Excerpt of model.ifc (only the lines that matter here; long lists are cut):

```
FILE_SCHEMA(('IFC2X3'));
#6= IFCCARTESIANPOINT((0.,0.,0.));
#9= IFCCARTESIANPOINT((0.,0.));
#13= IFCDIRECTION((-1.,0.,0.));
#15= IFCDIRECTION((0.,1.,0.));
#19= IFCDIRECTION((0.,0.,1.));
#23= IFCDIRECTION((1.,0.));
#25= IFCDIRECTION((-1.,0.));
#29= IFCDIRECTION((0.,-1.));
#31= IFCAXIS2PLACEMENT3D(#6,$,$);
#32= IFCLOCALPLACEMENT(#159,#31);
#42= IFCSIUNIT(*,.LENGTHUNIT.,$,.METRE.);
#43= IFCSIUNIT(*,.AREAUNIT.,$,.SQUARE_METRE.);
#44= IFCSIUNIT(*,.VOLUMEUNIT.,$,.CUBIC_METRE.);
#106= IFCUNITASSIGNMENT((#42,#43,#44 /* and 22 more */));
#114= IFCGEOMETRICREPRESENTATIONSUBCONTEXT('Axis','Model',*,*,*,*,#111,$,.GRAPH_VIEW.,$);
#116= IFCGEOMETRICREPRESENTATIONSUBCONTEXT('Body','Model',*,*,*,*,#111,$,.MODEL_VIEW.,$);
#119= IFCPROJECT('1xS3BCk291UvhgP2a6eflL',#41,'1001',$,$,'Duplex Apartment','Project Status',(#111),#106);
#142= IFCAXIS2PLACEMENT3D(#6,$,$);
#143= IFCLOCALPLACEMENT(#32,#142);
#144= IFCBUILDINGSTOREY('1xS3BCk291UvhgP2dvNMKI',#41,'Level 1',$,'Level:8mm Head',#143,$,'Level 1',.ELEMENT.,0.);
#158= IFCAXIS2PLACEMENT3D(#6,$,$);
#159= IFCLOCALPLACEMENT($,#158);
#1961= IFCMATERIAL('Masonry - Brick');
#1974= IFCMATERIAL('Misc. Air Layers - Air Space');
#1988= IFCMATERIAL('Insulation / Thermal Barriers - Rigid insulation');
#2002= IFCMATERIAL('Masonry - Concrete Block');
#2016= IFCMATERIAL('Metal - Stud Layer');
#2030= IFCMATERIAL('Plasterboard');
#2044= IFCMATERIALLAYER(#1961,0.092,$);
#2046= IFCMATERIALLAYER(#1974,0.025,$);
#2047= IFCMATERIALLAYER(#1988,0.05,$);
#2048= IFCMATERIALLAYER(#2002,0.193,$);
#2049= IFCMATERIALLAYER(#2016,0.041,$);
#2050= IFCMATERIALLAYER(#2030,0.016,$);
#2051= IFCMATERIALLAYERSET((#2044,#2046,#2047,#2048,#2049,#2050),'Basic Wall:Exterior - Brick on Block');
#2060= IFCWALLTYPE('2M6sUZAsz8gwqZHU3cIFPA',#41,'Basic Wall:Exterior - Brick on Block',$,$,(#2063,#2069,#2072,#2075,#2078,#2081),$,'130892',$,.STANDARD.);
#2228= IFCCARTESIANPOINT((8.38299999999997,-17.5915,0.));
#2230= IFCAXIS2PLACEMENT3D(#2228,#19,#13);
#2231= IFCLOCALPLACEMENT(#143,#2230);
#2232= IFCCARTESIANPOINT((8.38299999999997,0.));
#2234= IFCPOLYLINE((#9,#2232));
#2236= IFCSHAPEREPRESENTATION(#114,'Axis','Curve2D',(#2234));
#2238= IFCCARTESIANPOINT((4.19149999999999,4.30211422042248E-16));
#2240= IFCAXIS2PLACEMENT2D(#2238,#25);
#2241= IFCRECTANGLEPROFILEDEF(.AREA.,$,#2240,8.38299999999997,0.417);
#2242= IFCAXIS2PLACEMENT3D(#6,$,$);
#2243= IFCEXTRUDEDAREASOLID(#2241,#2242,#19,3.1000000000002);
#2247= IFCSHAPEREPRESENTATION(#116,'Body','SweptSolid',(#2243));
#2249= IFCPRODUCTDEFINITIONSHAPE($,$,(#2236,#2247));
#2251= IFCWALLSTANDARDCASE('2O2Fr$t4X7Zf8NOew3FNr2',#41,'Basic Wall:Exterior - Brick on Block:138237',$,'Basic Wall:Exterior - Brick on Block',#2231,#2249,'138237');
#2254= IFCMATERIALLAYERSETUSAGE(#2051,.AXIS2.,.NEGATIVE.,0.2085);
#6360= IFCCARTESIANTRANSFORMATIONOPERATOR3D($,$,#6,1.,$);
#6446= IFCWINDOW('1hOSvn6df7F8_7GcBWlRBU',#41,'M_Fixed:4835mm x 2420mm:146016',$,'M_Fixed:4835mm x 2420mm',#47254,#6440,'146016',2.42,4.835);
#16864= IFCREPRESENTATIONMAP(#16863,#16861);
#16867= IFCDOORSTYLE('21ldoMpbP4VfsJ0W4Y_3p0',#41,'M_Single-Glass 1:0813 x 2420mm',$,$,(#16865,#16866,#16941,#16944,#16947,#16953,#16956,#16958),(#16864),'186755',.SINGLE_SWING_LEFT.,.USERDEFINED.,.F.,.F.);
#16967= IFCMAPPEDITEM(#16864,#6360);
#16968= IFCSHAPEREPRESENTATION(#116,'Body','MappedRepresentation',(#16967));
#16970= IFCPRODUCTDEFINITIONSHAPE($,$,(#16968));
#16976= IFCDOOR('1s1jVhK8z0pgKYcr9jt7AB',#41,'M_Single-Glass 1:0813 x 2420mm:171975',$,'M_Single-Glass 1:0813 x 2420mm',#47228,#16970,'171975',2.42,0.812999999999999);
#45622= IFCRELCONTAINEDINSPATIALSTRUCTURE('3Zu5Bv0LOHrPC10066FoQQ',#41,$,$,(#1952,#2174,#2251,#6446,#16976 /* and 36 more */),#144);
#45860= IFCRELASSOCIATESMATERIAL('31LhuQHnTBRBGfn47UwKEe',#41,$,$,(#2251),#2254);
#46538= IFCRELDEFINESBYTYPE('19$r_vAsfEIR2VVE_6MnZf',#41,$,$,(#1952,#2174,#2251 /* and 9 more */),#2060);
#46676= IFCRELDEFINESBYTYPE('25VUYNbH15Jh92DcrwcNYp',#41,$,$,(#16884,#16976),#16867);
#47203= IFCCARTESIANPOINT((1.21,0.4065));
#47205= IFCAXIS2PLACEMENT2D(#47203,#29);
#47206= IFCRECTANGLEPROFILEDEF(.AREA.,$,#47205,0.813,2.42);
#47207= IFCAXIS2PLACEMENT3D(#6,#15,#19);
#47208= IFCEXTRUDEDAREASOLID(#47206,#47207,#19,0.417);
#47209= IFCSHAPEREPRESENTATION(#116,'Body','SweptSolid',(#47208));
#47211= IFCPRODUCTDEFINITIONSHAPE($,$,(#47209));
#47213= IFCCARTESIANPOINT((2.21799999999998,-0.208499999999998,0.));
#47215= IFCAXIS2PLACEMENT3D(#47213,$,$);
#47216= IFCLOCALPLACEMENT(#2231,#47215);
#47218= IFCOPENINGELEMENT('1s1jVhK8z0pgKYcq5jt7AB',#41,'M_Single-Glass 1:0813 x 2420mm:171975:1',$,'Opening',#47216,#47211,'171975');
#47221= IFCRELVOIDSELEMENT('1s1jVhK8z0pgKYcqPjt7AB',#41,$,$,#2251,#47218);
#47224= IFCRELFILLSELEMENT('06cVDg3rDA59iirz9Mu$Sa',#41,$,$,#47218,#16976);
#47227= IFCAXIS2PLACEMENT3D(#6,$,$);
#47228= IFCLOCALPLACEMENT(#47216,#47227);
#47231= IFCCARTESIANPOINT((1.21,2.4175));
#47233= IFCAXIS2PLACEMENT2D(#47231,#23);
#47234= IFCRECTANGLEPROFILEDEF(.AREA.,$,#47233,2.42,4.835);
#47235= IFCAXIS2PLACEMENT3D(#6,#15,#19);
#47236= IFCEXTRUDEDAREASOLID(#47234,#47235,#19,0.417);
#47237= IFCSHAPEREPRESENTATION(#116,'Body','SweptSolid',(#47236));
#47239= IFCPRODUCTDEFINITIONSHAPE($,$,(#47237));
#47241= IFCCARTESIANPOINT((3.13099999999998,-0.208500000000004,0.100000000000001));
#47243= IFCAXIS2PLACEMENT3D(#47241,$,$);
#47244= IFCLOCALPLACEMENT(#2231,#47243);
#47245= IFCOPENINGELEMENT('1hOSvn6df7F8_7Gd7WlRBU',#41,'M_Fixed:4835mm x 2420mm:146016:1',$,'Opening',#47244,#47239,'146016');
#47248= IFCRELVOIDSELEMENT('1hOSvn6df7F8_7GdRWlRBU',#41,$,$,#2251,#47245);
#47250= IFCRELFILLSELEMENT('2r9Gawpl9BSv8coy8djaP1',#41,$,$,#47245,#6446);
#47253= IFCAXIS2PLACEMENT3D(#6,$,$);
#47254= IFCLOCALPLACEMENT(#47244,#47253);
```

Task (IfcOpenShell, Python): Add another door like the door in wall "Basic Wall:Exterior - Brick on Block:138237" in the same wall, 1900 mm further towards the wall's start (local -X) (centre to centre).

```python
import ifcopenshell
import ifcopenshell.api.feature
import ifcopenshell.api.geometry
import ifcopenshell.api.root
import ifcopenshell.geom
import ifcopenshell.util.element
import ifcopenshell.util.placement
import ifcopenshell.util.shape

model = ifcopenshell.open("model.ifc")
settings = ifcopenshell.geom.settings()


def volume(element):
    """Net volume in cubic metres, openings subtracted."""
    shape = ifcopenshell.geom.create_shape(settings, element)
    return ifcopenshell.util.shape.get_volume(shape.geometry)


def reuse_history(source, copy):
    """copy_class also copies each property set's owner history, people and application; keep the originals."""
    for rel in copy.IsDefinedBy:
        if rel.is_a("IfcRelDefinesByProperties") and (history := rel.RelatingPropertyDefinition.OwnerHistory):
            rel.RelatingPropertyDefinition.OwnerHistory = source.OwnerHistory
            ifcopenshell.util.element.remove_deep2(model, history)


door = model.by_id(16976)
opening = door.FillsVoids[0].RelatingOpeningElement
wall = opening.VoidsElements[0].RelatingBuildingElement
before = volume(wall)
shift = ifcopenshell.util.placement.get_local_placement(wall.ObjectPlacement)[:3, 0] * -1.9

# copy_class copies the void relationship, type, container and properties, but no geometry.
new_opening = ifcopenshell.api.root.copy_class(model, product=opening)
new_opening.Representation = ifcopenshell.util.element.copy_deep(
    model, opening.Representation, exclude=["IfcGeometricRepresentationContext", "IfcRepresentationMap"]
)
new_opening.Name = "M_Single-Glass 1:0813 x 2420mm"
new_opening.Tag = None
new_door = ifcopenshell.api.root.copy_class(model, product=door)
new_door.Representation = ifcopenshell.util.element.copy_deep(
    model, door.Representation, exclude=["IfcGeometricRepresentationContext", "IfcRepresentationMap"]
)
new_door.Name = "M_Single-Glass 1:0813 x 2420mm"
new_door.Tag = None
reuse_history(door, new_door)
fills = ifcopenshell.api.feature.add_filling(model, opening=new_opening, element=new_door)
fills.OwnerHistory = new_door.OwnerHistory  # required in IFC2X3

for old, new in ((opening, new_opening), (door, new_door)):
    matrix = ifcopenshell.util.placement.get_local_placement(old.ObjectPlacement)
    matrix[:3, 3] += shift
    ifcopenshell.api.geometry.edit_object_placement(model, product=new, matrix=matrix, is_si=False)

after = volume(wall)

print(f"wall volume {before:.3f} -> {after:.3f} m3")

model.write("model_edited.ifc")
```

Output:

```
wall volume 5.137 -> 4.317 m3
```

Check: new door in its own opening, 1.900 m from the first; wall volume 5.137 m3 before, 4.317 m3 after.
